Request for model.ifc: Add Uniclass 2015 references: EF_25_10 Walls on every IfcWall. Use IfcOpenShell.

First a look at what the model holds.

```python
import ifcopenshell

model = ifcopenshell.open("model.ifc")
print(model.schema)
print("classifications:", [c.Name for c in model.by_type("IfcClassification")])
for ifc_class in ("IfcDoor", "IfcRoof", "IfcStair", "IfcWall", "IfcWindow"):
    print(ifc_class, len(model.by_type(ifc_class)))
```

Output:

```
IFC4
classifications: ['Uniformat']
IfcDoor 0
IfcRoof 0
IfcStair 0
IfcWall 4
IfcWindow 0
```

```python
import ifcopenshell
import ifcopenshell.api.classification

model = ifcopenshell.open("model.ifc")

system = ifcopenshell.api.classification.add_classification(model, classification="Uniclass 2015")

codes = {
    "IfcWall": ("EF_25_10", "Walls"),
}
for ifc_class, (code, name) in codes.items():
    products = model.by_type(ifc_class)
    ifcopenshell.api.classification.add_reference(
        model, products=products, classification=system, identification=code, name=name
    )
    print(code, len(products))

model.write("model_rev.ifc")
```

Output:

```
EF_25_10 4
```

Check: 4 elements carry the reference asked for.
